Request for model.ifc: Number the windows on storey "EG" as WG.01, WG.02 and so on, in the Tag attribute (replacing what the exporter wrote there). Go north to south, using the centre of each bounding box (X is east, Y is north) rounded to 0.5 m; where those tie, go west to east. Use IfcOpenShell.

First a look at what the model holds.

```python
import ifcopenshell
import ifcopenshell.util.element
import ifcopenshell.util.placement

model = ifcopenshell.open("model.ifc")
print(model.schema)
storey = next(s for s in model.by_type("IfcBuildingStorey") if s.Name == "EG")
windows = [e for e in ifcopenshell.util.element.get_decomposition(storey) if e.is_a("IfcWindow")]
for e in sorted(windows, key=lambda e: e.id()):
    origin = ifcopenshell.util.placement.get_local_placement(e.ObjectPlacement)[:3, 3]
    print(e.id(), e.Tag, e.Name, origin.round(2) + 0.0, sep=" | ")
```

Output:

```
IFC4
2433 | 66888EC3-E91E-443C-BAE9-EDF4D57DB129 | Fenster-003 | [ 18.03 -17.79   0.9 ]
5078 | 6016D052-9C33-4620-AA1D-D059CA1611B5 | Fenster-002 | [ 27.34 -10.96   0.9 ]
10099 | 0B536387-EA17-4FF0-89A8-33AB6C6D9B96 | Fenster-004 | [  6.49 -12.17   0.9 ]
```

```python
import ifcopenshell
import ifcopenshell.geom
import ifcopenshell.util.element
import ifcopenshell.util.shape

model = ifcopenshell.open("model.ifc")
settings = ifcopenshell.geom.settings()
settings.set("use-world-coords", True)


def centre(element):
    shape = ifcopenshell.geom.create_shape(settings, element)
    return ifcopenshell.util.shape.get_bbox_centroid(shape.geometry)


storey = next(s for s in model.by_type("IfcBuildingStorey") if s.Name == "EG")
windows = [e for e in ifcopenshell.util.element.get_decomposition(storey) if e.is_a("IfcWindow")]

# Insertion points can sit at a corner or the storey origin, so sort by the geometry (in metres).
centres = {e: centre(e) for e in windows}
windows.sort(key=lambda e: (-round(centres[e][1] / 0.5), centres[e][0]))

for i, e in enumerate(windows, start=1):
    number = f"WG.{i:02d}"
    e.Tag = number
    print(e.id(), number)

model.write("model_rev.ifc")
```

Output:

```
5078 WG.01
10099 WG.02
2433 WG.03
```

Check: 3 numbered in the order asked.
